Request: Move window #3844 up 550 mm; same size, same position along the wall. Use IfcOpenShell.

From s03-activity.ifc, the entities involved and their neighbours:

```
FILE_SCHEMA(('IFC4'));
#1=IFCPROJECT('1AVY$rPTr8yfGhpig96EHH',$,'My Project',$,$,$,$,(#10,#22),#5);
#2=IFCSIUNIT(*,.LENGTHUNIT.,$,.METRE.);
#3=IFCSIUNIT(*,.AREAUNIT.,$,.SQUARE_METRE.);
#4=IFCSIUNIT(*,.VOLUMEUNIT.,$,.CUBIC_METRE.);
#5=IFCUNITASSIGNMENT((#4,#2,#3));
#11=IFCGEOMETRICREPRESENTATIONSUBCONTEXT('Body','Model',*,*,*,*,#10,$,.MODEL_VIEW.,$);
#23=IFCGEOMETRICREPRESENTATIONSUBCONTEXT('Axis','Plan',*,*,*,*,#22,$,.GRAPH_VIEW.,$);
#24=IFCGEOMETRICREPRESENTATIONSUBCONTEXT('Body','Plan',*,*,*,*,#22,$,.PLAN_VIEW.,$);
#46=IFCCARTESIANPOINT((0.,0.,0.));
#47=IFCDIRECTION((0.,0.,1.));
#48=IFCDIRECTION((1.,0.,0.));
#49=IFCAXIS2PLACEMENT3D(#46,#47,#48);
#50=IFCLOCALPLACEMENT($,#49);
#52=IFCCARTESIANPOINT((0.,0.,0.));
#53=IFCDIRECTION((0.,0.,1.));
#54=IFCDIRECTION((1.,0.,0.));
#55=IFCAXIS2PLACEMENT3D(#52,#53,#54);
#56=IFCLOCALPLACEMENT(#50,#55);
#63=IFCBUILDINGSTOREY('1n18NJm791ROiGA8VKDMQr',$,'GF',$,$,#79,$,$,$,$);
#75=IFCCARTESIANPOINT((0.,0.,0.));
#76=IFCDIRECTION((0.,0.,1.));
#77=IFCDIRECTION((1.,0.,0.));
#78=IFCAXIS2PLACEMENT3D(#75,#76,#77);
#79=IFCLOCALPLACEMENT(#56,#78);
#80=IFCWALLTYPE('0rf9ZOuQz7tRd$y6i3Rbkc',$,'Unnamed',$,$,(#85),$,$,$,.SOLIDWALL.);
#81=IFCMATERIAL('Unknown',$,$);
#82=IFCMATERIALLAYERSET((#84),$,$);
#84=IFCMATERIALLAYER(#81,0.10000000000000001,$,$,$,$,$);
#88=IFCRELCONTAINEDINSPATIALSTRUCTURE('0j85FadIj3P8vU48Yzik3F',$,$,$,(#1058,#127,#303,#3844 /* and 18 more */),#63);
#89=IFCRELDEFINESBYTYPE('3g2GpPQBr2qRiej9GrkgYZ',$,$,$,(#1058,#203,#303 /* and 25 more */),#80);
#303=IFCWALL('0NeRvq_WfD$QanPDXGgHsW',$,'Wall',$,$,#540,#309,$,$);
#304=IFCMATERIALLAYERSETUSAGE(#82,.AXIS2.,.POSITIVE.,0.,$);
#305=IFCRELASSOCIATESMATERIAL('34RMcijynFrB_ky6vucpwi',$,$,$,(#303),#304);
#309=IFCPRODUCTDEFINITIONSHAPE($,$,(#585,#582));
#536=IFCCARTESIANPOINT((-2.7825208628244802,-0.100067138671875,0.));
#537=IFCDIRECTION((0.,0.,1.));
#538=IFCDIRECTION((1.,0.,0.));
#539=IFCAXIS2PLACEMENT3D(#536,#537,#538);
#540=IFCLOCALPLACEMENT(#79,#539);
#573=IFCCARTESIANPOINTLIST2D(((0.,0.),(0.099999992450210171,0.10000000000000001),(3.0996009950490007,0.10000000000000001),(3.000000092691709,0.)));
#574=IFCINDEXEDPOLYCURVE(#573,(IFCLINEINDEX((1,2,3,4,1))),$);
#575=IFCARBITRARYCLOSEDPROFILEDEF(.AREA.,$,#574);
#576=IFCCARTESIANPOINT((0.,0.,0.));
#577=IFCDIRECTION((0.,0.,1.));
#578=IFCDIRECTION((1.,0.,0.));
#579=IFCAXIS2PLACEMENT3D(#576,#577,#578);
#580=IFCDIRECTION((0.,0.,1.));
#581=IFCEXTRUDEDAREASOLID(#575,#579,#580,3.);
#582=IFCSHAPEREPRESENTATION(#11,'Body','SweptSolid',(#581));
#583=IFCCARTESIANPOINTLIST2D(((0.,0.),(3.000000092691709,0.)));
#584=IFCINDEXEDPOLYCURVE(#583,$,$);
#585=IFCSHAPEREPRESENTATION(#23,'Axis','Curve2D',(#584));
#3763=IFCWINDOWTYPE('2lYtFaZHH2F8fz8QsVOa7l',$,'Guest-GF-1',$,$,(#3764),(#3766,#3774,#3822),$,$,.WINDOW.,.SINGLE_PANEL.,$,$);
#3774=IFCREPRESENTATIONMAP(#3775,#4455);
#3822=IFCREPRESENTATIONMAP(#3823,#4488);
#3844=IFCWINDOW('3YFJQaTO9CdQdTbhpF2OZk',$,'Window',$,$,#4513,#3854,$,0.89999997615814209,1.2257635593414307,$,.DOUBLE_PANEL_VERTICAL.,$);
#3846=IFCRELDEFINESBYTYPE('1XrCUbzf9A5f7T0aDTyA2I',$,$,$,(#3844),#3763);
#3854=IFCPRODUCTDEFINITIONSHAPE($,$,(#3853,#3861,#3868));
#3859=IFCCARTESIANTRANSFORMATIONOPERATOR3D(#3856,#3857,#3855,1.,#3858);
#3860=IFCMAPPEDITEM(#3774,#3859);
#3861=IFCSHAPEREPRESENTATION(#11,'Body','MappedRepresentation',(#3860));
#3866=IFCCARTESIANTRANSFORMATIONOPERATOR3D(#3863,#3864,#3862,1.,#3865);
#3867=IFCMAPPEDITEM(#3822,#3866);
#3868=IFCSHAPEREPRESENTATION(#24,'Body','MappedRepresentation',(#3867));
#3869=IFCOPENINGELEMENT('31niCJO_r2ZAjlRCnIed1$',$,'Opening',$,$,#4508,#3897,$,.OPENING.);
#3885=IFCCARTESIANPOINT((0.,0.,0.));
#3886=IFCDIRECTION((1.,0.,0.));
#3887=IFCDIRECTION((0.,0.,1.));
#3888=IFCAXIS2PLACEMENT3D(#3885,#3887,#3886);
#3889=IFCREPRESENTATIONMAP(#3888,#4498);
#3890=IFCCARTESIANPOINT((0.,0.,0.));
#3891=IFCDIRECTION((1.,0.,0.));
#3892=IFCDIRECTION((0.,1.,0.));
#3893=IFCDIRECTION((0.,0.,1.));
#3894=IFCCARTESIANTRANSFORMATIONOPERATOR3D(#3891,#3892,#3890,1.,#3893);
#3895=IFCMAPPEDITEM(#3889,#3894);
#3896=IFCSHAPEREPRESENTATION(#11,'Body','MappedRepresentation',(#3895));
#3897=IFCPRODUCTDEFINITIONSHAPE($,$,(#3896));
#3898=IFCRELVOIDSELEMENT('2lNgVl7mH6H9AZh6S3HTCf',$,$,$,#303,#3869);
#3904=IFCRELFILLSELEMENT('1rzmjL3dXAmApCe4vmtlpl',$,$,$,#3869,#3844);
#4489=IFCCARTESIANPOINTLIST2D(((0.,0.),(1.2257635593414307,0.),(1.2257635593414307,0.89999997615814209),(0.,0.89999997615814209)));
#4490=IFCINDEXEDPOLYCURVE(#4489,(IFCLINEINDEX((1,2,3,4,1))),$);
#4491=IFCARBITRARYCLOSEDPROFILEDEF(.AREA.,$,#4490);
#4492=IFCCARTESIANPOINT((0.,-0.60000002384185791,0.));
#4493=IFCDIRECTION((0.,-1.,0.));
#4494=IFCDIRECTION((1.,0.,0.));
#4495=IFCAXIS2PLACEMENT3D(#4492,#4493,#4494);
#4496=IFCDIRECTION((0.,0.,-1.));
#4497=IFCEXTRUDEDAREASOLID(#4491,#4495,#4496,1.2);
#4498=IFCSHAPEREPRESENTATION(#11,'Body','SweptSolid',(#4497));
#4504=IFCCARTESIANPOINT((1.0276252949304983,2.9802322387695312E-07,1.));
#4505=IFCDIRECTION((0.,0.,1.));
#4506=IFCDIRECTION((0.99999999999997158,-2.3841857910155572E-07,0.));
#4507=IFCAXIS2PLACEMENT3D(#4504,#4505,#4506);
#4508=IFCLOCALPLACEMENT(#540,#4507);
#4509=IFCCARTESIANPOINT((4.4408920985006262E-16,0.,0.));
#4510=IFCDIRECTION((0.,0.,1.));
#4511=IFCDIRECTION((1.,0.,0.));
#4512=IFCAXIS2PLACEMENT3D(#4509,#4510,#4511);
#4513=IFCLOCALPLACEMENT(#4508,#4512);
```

```python
import numpy as np
import ifcopenshell
import ifcopenshell.api.geometry
import ifcopenshell.util.placement
import ifcopenshell.util.unit

model = ifcopenshell.open("s03-activity.ifc")
unit_scale = ifcopenshell.util.unit.calculate_unit_scale(model)

window = model.by_guid("3YFJQaTO9CdQdTbhpF2OZk")
opening = window.FillsVoids[0].RelatingOpeningElement
dz = 0.55 / unit_scale

shift = np.array([0.0, 0.0, dz])
# The window is placed relative to its opening, so it follows when the opening moves.
matrix = ifcopenshell.util.placement.get_local_placement(opening.ObjectPlacement)
matrix[:3, 3] += shift
ifcopenshell.api.geometry.edit_object_placement(
    model, product=opening, matrix=matrix, is_si=False, should_transform_children=True
)

print(f"moved by {dz * unit_scale:+.3f} m")

model.write("s03-activity_rev.ifc")
```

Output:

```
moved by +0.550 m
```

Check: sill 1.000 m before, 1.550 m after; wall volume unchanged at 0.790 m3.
